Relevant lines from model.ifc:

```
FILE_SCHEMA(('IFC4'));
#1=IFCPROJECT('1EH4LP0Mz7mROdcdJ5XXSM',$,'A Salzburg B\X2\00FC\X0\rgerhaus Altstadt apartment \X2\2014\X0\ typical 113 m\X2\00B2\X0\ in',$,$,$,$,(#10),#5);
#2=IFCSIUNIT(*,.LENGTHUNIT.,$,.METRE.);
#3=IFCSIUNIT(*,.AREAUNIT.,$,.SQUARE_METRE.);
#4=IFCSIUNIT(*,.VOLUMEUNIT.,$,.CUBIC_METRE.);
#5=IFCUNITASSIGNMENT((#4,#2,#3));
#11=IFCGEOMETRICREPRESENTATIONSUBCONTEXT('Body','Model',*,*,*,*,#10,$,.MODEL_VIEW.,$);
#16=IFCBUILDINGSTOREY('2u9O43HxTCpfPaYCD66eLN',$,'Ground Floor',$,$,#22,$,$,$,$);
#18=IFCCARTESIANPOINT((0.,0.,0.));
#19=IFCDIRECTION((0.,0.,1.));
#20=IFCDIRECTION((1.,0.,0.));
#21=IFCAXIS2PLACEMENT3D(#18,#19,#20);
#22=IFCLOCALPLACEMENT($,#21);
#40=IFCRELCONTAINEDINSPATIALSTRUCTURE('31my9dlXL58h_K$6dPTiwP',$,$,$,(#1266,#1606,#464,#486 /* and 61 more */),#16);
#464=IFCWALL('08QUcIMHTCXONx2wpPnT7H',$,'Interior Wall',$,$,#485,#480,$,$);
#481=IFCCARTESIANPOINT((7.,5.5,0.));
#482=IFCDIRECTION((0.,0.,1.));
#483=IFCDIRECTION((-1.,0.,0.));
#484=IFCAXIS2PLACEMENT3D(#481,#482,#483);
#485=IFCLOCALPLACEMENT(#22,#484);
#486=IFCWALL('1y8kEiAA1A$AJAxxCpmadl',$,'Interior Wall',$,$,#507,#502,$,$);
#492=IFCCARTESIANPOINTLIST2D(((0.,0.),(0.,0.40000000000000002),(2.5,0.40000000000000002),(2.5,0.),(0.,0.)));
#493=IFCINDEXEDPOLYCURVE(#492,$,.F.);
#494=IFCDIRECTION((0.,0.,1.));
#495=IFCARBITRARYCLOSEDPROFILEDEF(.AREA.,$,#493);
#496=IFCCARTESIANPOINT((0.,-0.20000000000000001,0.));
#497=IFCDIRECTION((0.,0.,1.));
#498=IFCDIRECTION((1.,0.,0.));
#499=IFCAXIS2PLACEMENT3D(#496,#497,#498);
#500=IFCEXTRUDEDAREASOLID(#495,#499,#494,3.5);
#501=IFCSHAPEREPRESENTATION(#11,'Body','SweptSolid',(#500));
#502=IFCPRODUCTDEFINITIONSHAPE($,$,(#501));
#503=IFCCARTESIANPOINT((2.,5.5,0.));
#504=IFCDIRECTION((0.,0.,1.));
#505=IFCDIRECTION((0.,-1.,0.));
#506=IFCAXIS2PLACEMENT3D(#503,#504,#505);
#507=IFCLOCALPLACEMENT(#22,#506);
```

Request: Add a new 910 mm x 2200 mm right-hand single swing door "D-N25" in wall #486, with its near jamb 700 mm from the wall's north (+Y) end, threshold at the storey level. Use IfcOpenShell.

```python
import numpy as np
import ifcopenshell
import ifcopenshell.api.feature
import ifcopenshell.api.geometry
import ifcopenshell.api.root
import ifcopenshell.api.spatial
import ifcopenshell.geom
import ifcopenshell.util.element
import ifcopenshell.util.placement
import ifcopenshell.util.representation
import ifcopenshell.util.shape
import ifcopenshell.util.unit

model = ifcopenshell.open("model.ifc")
unit_scale = ifcopenshell.util.unit.calculate_unit_scale(model)
settings = ifcopenshell.geom.settings()


def volume(element):
    """Net volume in cubic metres, openings subtracted."""
    shape = ifcopenshell.geom.create_shape(settings, element)
    return ifcopenshell.util.shape.get_volume(shape.geometry)


wall = model.by_guid("1y8kEiAA1A$AJAxxCpmadl")
storey = ifcopenshell.util.element.get_container(wall, ifc_class="IfcBuildingStorey")
context = ifcopenshell.util.representation.get_context(model, "Model", "Body", "MODEL_VIEW")
before = volume(wall)

width, height, from_end, sill = 0.91, 2.2, 0.7, 0.0  # metres

# The wall runs along its own X axis, and the end named is its -X end.
wall_shape = ifcopenshell.geom.create_shape(settings, wall)
x, y, z = ifcopenshell.util.shape.get_vertices(wall_shape.geometry).T
start = x.min() + from_end
face, thickness = float(y.min()), float(y.max() - y.min())
wall_matrix = ifcopenshell.util.placement.get_local_placement(wall.ObjectPlacement)
level = ifcopenshell.util.placement.get_local_placement(storey.ObjectPlacement)[2, 3]


def in_wall(x, y):
    """Placement at x, y metres in the wall's axes, at sill height."""
    matrix = wall_matrix.copy()
    matrix[:, 3] = wall_matrix @ np.array([x / unit_scale, y / unit_scale, 0.0, 1.0])
    matrix[2, 3] = level + sill / unit_scale
    return matrix


# Opening: a box that overshoots both wall faces by 50 mm.
opening = ifcopenshell.api.root.create_entity(model, ifc_class="IfcOpeningElement", predefined_type="OPENING")
box = ifcopenshell.api.geometry.add_wall_representation(
    model, context=context, length=width, height=height, thickness=thickness + 0.1
)
ifcopenshell.api.geometry.assign_representation(model, product=opening, representation=box)
ifcopenshell.api.geometry.edit_object_placement(model, product=opening, matrix=in_wall(start, face - 0.05), is_si=False)
ifcopenshell.api.feature.add_feature(model, feature=opening, element=wall)

door = ifcopenshell.api.root.create_entity(model, ifc_class="IfcDoor", name="D-N25", predefined_type="DOOR")
door.OverallWidth, door.OverallHeight = width / unit_scale, height / unit_scale
door.OperationType = "SINGLE_SWING_RIGHT"
body = ifcopenshell.api.geometry.add_door_representation(
    model,
    context=context,
    overall_width=door.OverallWidth,
    overall_height=door.OverallHeight,
    operation_type="SINGLE_SWING_RIGHT",
    lining_properties={"LiningDepth": thickness / unit_scale, "ThresholdDepth": thickness / unit_scale},
)
ifcopenshell.api.geometry.assign_representation(model, product=door, representation=body)
ifcopenshell.api.spatial.assign_container(model, products=[door], relating_structure=storey)
ifcopenshell.api.feature.add_filling(model, opening=opening, element=door)

# The lining spans the wall, so the door starts at the wall face.
ifcopenshell.api.geometry.edit_object_placement(model, product=door, matrix=in_wall(start, face), is_si=False)

after = volume(wall)

print(f"wall volume {before:.3f} -> {after:.3f} m3")

model.write("model_v2.ifc")
```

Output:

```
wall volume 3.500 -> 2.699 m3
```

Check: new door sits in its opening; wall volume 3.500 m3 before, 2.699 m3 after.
